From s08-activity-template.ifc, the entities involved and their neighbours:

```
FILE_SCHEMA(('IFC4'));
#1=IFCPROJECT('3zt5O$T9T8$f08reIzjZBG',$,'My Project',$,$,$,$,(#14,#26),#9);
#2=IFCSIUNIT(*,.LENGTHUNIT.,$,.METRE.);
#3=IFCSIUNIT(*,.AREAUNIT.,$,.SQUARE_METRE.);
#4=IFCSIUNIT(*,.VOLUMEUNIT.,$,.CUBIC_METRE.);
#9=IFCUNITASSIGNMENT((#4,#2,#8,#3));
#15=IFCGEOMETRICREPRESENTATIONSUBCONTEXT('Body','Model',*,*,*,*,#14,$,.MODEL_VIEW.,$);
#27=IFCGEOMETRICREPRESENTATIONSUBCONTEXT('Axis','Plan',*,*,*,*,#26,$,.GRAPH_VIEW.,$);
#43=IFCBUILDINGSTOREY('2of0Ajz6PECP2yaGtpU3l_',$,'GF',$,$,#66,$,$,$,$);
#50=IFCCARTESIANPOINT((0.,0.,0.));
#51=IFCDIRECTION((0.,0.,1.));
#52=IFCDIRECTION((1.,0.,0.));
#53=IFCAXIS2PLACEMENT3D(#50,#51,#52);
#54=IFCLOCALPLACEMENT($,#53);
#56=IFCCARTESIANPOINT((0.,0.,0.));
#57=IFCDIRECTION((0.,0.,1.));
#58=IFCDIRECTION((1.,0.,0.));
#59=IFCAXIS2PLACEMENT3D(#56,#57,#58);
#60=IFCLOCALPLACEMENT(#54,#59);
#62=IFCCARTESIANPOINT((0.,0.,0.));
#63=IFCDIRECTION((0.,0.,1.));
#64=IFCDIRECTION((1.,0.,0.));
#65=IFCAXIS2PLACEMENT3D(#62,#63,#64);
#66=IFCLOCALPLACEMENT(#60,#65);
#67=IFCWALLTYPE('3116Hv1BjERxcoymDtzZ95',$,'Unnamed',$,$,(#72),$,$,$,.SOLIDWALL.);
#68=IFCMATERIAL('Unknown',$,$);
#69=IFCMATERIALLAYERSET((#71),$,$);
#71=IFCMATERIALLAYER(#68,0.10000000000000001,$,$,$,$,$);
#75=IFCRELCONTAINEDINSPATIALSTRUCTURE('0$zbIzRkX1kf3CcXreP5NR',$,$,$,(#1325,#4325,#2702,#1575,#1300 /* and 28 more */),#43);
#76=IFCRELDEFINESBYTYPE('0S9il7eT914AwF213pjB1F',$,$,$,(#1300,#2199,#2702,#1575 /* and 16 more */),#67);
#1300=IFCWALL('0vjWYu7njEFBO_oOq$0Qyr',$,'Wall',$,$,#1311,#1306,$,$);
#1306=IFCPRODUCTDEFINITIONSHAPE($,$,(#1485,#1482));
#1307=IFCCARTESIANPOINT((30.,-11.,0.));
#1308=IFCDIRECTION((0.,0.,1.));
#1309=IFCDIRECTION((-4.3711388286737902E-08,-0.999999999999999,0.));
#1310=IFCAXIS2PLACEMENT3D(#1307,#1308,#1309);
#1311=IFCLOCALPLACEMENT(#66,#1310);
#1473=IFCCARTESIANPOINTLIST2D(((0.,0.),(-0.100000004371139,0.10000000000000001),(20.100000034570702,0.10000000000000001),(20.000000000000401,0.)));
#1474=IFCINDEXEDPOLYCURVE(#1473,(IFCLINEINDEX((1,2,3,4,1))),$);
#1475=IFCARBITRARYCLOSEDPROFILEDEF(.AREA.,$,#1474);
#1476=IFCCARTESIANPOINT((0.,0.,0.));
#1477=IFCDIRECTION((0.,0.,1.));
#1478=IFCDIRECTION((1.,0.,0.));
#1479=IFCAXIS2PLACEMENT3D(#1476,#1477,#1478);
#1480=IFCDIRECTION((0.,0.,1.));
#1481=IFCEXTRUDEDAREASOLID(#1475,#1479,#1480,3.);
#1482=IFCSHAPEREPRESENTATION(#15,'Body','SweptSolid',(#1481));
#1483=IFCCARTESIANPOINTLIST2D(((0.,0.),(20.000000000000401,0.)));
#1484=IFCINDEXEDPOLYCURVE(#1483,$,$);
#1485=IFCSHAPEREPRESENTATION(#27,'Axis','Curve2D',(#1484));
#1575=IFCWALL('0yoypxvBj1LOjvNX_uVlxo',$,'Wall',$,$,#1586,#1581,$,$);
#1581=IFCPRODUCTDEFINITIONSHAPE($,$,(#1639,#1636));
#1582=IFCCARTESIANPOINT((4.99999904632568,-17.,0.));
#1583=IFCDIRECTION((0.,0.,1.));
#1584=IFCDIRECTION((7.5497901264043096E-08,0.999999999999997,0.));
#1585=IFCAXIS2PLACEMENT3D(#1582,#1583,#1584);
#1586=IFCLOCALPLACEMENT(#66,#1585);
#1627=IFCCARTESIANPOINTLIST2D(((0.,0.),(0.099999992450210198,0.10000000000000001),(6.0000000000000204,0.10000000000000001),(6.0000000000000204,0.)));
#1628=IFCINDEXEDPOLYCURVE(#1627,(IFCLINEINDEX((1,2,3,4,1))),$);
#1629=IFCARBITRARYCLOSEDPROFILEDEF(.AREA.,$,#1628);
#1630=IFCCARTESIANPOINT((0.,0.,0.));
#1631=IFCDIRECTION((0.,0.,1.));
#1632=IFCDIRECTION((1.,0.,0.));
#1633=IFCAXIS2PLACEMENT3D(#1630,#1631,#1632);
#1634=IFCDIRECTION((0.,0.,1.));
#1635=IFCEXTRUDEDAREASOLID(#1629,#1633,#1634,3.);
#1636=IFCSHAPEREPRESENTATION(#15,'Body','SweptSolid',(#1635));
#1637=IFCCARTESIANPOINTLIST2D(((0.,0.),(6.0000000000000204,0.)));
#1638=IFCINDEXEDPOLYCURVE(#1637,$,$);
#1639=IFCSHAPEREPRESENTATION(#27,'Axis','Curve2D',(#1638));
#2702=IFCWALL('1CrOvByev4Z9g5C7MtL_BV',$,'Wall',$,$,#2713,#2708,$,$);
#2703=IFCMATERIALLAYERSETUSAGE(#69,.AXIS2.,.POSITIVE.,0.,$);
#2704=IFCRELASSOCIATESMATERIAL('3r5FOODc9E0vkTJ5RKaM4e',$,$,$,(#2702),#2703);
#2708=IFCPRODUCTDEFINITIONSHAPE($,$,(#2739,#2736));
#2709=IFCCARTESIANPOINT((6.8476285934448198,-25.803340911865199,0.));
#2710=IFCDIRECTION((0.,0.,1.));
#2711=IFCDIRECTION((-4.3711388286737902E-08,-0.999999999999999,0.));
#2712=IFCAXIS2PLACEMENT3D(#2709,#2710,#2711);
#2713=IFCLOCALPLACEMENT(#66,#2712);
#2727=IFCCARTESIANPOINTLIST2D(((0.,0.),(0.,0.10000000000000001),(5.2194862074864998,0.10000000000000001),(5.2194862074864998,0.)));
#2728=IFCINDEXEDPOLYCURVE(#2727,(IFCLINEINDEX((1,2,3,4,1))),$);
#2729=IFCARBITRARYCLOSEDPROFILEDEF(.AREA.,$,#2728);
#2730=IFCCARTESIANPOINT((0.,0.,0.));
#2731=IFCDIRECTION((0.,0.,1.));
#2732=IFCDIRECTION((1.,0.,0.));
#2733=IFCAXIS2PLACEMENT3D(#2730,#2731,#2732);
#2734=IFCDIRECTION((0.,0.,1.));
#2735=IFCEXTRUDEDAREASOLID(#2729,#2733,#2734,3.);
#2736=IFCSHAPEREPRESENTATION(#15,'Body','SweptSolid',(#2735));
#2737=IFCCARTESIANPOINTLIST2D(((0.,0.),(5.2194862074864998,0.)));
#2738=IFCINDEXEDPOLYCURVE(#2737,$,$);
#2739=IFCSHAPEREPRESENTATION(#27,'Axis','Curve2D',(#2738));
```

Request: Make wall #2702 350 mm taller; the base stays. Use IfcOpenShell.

```python
import ifcopenshell
import ifcopenshell.geom
import ifcopenshell.util.representation
import ifcopenshell.util.shape
import ifcopenshell.util.unit

model = ifcopenshell.open("s08-activity-template.ifc")
unit_scale = ifcopenshell.util.unit.calculate_unit_scale(model)
settings = ifcopenshell.geom.settings()


def volume(element):
    """Net volume in cubic metres, openings subtracted."""
    shape = ifcopenshell.geom.create_shape(settings, element)
    return ifcopenshell.util.shape.get_volume(shape.geometry)


wall = model.by_guid("1CrOvByev4Z9g5C7MtL_BV")
before = volume(wall)

body = ifcopenshell.util.representation.get_representation(wall, "Model", "Body")
solid = body.Items[0]
old_height = solid.Depth
solid.Depth += 0.35 / unit_scale
after = volume(wall)

print(f"height {old_height:g} -> {solid.Depth:g}, volume {before:.3f} -> {after:.3f} m3")

model.write("s08-activity-template_edited.ifc")
```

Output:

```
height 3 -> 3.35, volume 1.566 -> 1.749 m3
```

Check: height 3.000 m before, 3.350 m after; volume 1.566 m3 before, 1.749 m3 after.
